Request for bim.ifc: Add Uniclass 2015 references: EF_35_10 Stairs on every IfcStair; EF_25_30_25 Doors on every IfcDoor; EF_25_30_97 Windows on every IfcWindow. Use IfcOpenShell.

First a look at what the model holds.

```python
import ifcopenshell

model = ifcopenshell.open("bim.ifc")
print(model.schema)
print("classifications:", [c.Name for c in model.by_type("IfcClassification")])
for ifc_class in ("IfcDoor", "IfcRoof", "IfcStair", "IfcWall", "IfcWindow"):
    print(ifc_class, len(model.by_type(ifc_class)))
```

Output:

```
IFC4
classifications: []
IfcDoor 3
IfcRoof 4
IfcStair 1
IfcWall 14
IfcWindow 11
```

```python
import ifcopenshell
import ifcopenshell.api.classification

model = ifcopenshell.open("bim.ifc")

system = ifcopenshell.api.classification.add_classification(model, classification="Uniclass 2015")

codes = {
    "IfcStair": ("EF_35_10", "Stairs"),
    "IfcDoor": ("EF_25_30_25", "Doors"),
    "IfcWindow": ("EF_25_30_97", "Windows"),
}
for ifc_class, (code, name) in codes.items():
    products = model.by_type(ifc_class)
    ifcopenshell.api.classification.add_reference(
        model, products=products, classification=system, identification=code, name=name
    )
    print(code, len(products))

model.write("bim_edited.ifc")
```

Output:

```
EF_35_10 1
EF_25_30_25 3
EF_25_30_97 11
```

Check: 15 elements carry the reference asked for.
